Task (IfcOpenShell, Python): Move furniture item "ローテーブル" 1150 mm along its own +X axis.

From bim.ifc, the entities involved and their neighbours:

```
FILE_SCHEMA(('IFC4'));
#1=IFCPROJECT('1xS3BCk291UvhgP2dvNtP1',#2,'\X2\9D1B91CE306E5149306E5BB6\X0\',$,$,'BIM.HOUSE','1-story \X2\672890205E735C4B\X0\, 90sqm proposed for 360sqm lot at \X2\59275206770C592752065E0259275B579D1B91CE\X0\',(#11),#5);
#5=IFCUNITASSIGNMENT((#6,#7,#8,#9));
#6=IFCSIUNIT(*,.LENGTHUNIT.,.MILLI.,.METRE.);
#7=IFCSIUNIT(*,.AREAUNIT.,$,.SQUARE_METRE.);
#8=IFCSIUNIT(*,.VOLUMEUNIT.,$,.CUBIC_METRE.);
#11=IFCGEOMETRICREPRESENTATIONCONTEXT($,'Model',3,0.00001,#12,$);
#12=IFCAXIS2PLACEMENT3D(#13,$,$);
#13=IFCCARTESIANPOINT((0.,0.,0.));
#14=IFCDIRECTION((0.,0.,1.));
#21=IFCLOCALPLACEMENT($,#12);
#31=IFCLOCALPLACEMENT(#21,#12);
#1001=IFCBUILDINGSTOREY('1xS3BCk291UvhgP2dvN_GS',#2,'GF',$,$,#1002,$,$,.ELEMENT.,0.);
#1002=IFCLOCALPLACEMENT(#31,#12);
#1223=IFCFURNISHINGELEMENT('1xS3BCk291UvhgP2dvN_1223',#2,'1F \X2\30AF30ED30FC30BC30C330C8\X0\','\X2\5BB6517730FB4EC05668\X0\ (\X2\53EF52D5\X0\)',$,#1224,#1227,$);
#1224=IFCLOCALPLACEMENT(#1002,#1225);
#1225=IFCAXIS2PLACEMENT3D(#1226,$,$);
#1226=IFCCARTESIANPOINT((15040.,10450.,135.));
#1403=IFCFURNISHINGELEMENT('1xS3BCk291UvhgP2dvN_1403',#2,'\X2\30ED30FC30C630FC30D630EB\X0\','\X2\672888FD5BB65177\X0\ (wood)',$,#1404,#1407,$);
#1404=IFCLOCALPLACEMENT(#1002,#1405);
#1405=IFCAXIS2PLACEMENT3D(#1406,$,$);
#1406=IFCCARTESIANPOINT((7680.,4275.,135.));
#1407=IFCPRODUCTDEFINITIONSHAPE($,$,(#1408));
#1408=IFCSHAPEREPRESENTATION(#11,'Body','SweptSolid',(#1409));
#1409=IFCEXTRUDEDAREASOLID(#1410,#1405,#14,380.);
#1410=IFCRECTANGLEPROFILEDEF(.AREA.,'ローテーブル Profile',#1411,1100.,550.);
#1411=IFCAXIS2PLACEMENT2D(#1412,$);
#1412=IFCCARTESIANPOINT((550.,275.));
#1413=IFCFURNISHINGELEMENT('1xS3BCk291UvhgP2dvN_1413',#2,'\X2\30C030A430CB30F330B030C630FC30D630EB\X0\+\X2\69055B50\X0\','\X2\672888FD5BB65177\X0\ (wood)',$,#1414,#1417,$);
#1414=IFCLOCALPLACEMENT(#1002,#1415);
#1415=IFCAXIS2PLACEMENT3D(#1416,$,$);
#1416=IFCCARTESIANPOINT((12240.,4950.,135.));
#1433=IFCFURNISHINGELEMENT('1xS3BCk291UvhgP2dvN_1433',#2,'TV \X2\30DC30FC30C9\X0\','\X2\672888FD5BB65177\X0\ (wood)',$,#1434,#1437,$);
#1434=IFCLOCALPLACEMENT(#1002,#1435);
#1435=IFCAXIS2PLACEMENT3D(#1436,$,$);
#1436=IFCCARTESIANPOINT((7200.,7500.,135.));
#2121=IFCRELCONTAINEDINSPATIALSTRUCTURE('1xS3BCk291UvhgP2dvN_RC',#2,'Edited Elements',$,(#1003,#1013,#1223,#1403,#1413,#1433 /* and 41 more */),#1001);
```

```python
import ifcopenshell
import ifcopenshell.api.geometry
import ifcopenshell.util.placement

model = ifcopenshell.open("bim.ifc")

item = model.by_guid("1xS3BCk291UvhgP2dvN_1403")
matrix = ifcopenshell.util.placement.get_local_placement(item.ObjectPlacement)
matrix[:3, 3] += matrix[:3, 0] * 1150.0
ifcopenshell.api.geometry.edit_object_placement(model, product=item, matrix=matrix, is_si=False)

print(ifcopenshell.util.placement.get_local_placement(item.ObjectPlacement).round(3) + 0.0)

model.write("bim_v2.ifc")
```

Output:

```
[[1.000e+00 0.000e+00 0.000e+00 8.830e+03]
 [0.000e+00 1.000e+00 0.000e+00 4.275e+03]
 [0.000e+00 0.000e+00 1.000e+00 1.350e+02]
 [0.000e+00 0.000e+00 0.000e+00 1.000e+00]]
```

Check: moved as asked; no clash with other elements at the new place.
